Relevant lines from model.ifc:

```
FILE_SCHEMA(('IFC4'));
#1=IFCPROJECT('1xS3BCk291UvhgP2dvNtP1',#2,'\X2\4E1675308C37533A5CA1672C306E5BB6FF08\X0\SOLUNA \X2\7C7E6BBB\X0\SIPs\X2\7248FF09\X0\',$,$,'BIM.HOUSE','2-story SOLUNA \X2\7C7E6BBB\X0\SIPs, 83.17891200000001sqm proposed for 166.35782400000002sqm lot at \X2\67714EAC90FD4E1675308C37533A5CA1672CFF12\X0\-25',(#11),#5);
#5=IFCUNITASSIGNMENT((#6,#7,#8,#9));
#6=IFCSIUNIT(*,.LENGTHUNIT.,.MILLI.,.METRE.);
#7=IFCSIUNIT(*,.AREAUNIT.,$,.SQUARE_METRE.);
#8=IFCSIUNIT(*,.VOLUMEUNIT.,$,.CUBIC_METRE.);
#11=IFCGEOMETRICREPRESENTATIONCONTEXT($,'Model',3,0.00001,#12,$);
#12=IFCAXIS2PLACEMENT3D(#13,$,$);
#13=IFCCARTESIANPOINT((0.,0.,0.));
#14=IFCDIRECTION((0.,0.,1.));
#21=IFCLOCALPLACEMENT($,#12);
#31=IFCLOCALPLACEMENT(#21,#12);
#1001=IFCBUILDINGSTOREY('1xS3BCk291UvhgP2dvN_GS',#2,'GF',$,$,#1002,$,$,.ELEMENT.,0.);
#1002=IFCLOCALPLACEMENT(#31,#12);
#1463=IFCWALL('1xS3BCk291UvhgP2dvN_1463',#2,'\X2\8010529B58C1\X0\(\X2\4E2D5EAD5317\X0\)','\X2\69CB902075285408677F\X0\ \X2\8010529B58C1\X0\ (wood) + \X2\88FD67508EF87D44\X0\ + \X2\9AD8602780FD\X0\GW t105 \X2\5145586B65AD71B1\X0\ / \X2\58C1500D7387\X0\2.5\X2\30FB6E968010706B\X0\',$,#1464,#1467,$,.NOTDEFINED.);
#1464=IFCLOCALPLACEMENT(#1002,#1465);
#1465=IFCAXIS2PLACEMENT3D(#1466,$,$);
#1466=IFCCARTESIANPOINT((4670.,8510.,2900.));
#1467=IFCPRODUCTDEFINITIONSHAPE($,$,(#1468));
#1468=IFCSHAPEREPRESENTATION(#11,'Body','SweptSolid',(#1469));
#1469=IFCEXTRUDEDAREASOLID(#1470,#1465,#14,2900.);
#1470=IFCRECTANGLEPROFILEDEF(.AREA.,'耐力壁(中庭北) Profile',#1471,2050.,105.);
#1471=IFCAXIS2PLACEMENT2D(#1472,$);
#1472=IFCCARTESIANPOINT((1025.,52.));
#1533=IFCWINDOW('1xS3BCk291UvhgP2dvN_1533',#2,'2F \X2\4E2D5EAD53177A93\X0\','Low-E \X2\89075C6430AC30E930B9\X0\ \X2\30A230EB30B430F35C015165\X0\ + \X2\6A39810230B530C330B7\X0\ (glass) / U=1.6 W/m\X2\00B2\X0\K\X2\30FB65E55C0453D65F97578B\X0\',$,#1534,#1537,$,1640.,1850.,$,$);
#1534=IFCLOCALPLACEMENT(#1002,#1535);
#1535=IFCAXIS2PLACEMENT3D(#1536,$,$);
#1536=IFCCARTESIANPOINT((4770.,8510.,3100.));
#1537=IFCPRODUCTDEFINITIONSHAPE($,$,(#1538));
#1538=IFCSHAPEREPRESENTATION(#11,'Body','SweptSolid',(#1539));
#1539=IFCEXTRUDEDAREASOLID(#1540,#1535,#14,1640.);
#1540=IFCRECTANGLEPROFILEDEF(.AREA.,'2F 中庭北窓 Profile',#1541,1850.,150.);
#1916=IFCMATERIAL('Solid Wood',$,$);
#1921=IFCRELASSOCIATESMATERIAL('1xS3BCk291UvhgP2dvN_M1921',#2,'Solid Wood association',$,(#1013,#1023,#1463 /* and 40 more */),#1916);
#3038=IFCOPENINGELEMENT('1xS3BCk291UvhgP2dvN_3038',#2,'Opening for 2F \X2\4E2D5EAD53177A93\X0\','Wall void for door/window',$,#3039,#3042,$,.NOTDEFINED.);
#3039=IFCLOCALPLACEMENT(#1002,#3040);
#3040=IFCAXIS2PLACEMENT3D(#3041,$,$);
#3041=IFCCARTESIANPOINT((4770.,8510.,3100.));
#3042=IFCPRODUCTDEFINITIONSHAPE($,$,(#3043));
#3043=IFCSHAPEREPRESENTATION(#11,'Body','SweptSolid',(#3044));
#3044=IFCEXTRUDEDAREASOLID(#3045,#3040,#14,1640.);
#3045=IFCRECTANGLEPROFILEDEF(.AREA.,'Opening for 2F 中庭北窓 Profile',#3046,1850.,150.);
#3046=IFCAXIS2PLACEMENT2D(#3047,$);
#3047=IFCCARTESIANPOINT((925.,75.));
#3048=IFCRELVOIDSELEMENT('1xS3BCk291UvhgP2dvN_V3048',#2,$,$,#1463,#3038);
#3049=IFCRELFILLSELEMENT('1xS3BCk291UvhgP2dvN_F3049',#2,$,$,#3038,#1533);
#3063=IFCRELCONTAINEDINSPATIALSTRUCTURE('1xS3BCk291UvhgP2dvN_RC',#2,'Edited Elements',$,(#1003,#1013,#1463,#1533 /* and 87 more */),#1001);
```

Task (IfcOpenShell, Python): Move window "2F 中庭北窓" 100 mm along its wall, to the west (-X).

```python
import ifcopenshell
import ifcopenshell.api.geometry
import ifcopenshell.util.placement

model = ifcopenshell.open("model.ifc")

window = model.by_id(1533)
opening = window.FillsVoids[0].RelatingOpeningElement
wall = opening.VoidsElements[0].RelatingBuildingElement

wall_matrix = ifcopenshell.util.placement.get_local_placement(wall.ObjectPlacement)
shift = wall_matrix[:3, 0] * -100.0
before = ifcopenshell.util.placement.get_local_placement(window.ObjectPlacement)[:3, 3].copy()

# The window is not placed relative to its opening, so move both.
for product in (opening, window):
    matrix = ifcopenshell.util.placement.get_local_placement(product.ObjectPlacement)
    matrix[:3, 3] += shift
    ifcopenshell.api.geometry.edit_object_placement(model, product=product, matrix=matrix, is_si=False)

after = ifcopenshell.util.placement.get_local_placement(window.ObjectPlacement)[:3, 3]
print("window moved by", (after - before).round(3) + 0.0)

model.write("model_updated.ifc")
```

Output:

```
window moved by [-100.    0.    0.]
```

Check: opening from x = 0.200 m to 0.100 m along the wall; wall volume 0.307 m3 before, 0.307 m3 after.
